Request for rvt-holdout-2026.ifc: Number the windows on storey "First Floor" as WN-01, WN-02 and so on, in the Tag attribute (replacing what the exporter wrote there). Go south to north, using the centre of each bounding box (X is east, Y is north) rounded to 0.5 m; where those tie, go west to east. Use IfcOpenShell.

First a look at what the model holds.

```python
import ifcopenshell
import ifcopenshell.util.element
import ifcopenshell.util.placement

model = ifcopenshell.open("rvt-holdout-2026.ifc")
print(model.schema)
storey = next(s for s in model.by_type("IfcBuildingStorey") if s.Name == "First Floor")
windows = [e for e in ifcopenshell.util.element.get_decomposition(storey) if e.is_a("IfcWindow")]
for e in sorted(windows, key=lambda e: e.id()):
    origin = ifcopenshell.util.placement.get_local_placement(e.ObjectPlacement)[:3, 3]
    print(e.id(), e.Tag, e.Name, origin.round(2) + 0.0, sep=" | ")
```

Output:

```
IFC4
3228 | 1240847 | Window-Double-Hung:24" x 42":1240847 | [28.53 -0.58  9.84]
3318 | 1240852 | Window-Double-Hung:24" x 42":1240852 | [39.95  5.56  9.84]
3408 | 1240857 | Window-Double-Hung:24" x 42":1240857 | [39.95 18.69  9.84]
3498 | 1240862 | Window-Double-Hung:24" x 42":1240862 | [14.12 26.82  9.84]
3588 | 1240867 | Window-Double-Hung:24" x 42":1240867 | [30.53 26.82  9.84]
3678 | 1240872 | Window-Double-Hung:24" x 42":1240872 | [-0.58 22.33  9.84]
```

```python
import ifcopenshell
import ifcopenshell.geom
import ifcopenshell.util.element
import ifcopenshell.util.shape

model = ifcopenshell.open("rvt-holdout-2026.ifc")
settings = ifcopenshell.geom.settings()
settings.set("use-world-coords", True)


def centre(element):
    shape = ifcopenshell.geom.create_shape(settings, element)
    return ifcopenshell.util.shape.get_bbox_centroid(shape.geometry)


storey = next(s for s in model.by_type("IfcBuildingStorey") if s.Name == "First Floor")
windows = [e for e in ifcopenshell.util.element.get_decomposition(storey) if e.is_a("IfcWindow")]

# Insertion points can sit at a corner or the storey origin, so sort by the geometry (in metres).
centres = {e: centre(e) for e in windows}
windows.sort(key=lambda e: (round(centres[e][1] / 0.5), centres[e][0]))

for i, e in enumerate(windows, start=1):
    number = f"WN-{i:02d}"
    e.Tag = number
    print(e.id(), number)

model.write("rvt-holdout-2026_rev.ifc")
```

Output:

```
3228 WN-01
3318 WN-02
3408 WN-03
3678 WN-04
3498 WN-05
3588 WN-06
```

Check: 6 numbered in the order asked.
